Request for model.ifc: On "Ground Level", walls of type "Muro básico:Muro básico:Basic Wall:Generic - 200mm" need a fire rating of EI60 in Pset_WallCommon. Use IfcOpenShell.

First a look at what the model holds.

```python
import ifcopenshell
import ifcopenshell.util.element

model = ifcopenshell.open("model.ifc")
print(model.schema)
storey = next(s for s in model.by_type("IfcBuildingStorey") if s.Name == "Ground Level")
walls = [e for e in ifcopenshell.util.element.get_decomposition(storey) if e.is_a("IfcWall")]
seen = {}
for e in walls:
    element_type = ifcopenshell.util.element.get_type(e)
    key = (element_type.Name if element_type != e and element_type else None, ifcopenshell.util.element.get_pset(e, "Pset_WallCommon", "FireRating"))
    seen[key] = seen.get(key, 0) + 1
for (name, value), count in sorted(seen.items(), key=str):
    print(count, "x", name, "|", value)
```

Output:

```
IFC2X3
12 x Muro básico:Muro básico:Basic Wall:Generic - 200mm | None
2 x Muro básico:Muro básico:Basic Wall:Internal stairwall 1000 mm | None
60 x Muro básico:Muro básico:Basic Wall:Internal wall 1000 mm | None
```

```python
import ifcopenshell
import ifcopenshell.api.pset
import ifcopenshell.util.element

model = ifcopenshell.open("model.ifc")

storey = next(s for s in model.by_type("IfcBuildingStorey") if s.Name == "Ground Level")
walls = [e for e in ifcopenshell.util.element.get_decomposition(storey) if e.is_a("IfcWall")]

count = 0
for e in walls:
    element_type = ifcopenshell.util.element.get_type(e)
    if element_type in (None, e) or element_type.Name != "Muro básico:Muro básico:Basic Wall:Generic - 200mm":
        continue
    # add_pset returns the element's existing set when there is one.
    pset = ifcopenshell.api.pset.add_pset(model, product=e, name="Pset_WallCommon")
    ifcopenshell.api.pset.edit_pset(model, pset=pset, properties={"FireRating": "EI60"})
    count += 1

print(count, "walls updated")

model.write("model_edited.ifc")
```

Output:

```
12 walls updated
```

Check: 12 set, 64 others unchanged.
